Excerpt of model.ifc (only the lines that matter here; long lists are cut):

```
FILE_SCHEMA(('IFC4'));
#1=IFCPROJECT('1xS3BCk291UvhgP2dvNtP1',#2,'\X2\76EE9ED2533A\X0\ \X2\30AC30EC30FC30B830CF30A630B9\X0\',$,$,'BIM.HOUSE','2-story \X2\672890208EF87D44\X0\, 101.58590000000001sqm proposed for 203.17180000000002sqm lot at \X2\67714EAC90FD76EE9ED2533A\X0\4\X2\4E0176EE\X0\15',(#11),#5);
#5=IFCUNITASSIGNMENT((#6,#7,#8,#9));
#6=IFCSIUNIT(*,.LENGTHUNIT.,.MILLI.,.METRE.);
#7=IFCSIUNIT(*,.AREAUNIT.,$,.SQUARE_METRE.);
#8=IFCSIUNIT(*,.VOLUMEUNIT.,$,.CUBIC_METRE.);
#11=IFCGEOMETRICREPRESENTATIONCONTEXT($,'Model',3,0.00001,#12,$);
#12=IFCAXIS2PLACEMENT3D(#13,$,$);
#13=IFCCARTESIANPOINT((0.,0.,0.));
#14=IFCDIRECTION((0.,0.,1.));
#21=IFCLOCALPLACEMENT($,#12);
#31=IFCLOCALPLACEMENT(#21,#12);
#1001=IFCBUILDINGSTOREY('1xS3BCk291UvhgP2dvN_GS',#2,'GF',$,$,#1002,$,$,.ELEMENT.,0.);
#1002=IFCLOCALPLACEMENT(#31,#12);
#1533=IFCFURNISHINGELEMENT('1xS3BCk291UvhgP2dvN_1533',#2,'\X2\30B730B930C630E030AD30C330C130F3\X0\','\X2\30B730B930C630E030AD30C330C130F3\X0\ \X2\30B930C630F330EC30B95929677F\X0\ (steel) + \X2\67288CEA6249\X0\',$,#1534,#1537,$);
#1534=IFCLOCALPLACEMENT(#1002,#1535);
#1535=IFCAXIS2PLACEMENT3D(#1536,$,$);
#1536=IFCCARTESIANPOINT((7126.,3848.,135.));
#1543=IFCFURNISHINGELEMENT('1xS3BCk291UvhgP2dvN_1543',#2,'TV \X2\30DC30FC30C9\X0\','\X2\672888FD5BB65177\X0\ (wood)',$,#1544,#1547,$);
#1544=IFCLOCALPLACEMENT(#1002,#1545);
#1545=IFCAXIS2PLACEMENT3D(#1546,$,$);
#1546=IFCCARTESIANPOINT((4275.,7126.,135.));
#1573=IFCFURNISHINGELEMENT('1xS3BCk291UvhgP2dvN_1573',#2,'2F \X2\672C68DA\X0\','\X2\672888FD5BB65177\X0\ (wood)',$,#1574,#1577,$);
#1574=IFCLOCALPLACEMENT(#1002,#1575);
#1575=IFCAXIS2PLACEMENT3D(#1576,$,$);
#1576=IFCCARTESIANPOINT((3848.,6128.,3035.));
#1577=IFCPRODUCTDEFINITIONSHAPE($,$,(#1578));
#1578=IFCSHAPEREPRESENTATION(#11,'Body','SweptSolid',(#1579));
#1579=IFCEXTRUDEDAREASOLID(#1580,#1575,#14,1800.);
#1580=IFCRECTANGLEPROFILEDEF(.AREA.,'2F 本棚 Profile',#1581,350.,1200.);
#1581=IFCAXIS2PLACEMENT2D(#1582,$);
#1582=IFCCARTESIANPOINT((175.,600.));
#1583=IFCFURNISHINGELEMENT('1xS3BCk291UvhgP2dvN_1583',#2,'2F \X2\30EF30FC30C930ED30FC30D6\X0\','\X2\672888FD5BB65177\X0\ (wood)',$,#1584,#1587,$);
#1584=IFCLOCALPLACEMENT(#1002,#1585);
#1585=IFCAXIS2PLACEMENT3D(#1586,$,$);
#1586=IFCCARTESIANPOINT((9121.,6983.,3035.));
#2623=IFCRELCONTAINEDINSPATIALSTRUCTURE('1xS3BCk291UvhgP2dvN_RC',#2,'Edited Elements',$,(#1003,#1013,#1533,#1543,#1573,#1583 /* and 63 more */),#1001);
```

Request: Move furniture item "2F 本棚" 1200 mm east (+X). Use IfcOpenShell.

```python
import ifcopenshell
import ifcopenshell.api.geometry
import ifcopenshell.util.placement
import ifcopenshell.util.unit

model = ifcopenshell.open("model.ifc")
unit_scale = ifcopenshell.util.unit.calculate_unit_scale(model)

item = model.by_guid("1xS3BCk291UvhgP2dvN_1573")
matrix = ifcopenshell.util.placement.get_local_placement(item.ObjectPlacement)
matrix[0, 3] += 1.2 / unit_scale
ifcopenshell.api.geometry.edit_object_placement(model, product=item, matrix=matrix, is_si=False)

print(ifcopenshell.util.placement.get_local_placement(item.ObjectPlacement).round(3) + 0.0)

model.write("model-out.ifc")
```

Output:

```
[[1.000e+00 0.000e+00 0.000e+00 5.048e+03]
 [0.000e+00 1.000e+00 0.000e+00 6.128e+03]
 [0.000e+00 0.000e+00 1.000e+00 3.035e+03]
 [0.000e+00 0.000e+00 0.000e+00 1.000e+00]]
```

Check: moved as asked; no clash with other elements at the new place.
